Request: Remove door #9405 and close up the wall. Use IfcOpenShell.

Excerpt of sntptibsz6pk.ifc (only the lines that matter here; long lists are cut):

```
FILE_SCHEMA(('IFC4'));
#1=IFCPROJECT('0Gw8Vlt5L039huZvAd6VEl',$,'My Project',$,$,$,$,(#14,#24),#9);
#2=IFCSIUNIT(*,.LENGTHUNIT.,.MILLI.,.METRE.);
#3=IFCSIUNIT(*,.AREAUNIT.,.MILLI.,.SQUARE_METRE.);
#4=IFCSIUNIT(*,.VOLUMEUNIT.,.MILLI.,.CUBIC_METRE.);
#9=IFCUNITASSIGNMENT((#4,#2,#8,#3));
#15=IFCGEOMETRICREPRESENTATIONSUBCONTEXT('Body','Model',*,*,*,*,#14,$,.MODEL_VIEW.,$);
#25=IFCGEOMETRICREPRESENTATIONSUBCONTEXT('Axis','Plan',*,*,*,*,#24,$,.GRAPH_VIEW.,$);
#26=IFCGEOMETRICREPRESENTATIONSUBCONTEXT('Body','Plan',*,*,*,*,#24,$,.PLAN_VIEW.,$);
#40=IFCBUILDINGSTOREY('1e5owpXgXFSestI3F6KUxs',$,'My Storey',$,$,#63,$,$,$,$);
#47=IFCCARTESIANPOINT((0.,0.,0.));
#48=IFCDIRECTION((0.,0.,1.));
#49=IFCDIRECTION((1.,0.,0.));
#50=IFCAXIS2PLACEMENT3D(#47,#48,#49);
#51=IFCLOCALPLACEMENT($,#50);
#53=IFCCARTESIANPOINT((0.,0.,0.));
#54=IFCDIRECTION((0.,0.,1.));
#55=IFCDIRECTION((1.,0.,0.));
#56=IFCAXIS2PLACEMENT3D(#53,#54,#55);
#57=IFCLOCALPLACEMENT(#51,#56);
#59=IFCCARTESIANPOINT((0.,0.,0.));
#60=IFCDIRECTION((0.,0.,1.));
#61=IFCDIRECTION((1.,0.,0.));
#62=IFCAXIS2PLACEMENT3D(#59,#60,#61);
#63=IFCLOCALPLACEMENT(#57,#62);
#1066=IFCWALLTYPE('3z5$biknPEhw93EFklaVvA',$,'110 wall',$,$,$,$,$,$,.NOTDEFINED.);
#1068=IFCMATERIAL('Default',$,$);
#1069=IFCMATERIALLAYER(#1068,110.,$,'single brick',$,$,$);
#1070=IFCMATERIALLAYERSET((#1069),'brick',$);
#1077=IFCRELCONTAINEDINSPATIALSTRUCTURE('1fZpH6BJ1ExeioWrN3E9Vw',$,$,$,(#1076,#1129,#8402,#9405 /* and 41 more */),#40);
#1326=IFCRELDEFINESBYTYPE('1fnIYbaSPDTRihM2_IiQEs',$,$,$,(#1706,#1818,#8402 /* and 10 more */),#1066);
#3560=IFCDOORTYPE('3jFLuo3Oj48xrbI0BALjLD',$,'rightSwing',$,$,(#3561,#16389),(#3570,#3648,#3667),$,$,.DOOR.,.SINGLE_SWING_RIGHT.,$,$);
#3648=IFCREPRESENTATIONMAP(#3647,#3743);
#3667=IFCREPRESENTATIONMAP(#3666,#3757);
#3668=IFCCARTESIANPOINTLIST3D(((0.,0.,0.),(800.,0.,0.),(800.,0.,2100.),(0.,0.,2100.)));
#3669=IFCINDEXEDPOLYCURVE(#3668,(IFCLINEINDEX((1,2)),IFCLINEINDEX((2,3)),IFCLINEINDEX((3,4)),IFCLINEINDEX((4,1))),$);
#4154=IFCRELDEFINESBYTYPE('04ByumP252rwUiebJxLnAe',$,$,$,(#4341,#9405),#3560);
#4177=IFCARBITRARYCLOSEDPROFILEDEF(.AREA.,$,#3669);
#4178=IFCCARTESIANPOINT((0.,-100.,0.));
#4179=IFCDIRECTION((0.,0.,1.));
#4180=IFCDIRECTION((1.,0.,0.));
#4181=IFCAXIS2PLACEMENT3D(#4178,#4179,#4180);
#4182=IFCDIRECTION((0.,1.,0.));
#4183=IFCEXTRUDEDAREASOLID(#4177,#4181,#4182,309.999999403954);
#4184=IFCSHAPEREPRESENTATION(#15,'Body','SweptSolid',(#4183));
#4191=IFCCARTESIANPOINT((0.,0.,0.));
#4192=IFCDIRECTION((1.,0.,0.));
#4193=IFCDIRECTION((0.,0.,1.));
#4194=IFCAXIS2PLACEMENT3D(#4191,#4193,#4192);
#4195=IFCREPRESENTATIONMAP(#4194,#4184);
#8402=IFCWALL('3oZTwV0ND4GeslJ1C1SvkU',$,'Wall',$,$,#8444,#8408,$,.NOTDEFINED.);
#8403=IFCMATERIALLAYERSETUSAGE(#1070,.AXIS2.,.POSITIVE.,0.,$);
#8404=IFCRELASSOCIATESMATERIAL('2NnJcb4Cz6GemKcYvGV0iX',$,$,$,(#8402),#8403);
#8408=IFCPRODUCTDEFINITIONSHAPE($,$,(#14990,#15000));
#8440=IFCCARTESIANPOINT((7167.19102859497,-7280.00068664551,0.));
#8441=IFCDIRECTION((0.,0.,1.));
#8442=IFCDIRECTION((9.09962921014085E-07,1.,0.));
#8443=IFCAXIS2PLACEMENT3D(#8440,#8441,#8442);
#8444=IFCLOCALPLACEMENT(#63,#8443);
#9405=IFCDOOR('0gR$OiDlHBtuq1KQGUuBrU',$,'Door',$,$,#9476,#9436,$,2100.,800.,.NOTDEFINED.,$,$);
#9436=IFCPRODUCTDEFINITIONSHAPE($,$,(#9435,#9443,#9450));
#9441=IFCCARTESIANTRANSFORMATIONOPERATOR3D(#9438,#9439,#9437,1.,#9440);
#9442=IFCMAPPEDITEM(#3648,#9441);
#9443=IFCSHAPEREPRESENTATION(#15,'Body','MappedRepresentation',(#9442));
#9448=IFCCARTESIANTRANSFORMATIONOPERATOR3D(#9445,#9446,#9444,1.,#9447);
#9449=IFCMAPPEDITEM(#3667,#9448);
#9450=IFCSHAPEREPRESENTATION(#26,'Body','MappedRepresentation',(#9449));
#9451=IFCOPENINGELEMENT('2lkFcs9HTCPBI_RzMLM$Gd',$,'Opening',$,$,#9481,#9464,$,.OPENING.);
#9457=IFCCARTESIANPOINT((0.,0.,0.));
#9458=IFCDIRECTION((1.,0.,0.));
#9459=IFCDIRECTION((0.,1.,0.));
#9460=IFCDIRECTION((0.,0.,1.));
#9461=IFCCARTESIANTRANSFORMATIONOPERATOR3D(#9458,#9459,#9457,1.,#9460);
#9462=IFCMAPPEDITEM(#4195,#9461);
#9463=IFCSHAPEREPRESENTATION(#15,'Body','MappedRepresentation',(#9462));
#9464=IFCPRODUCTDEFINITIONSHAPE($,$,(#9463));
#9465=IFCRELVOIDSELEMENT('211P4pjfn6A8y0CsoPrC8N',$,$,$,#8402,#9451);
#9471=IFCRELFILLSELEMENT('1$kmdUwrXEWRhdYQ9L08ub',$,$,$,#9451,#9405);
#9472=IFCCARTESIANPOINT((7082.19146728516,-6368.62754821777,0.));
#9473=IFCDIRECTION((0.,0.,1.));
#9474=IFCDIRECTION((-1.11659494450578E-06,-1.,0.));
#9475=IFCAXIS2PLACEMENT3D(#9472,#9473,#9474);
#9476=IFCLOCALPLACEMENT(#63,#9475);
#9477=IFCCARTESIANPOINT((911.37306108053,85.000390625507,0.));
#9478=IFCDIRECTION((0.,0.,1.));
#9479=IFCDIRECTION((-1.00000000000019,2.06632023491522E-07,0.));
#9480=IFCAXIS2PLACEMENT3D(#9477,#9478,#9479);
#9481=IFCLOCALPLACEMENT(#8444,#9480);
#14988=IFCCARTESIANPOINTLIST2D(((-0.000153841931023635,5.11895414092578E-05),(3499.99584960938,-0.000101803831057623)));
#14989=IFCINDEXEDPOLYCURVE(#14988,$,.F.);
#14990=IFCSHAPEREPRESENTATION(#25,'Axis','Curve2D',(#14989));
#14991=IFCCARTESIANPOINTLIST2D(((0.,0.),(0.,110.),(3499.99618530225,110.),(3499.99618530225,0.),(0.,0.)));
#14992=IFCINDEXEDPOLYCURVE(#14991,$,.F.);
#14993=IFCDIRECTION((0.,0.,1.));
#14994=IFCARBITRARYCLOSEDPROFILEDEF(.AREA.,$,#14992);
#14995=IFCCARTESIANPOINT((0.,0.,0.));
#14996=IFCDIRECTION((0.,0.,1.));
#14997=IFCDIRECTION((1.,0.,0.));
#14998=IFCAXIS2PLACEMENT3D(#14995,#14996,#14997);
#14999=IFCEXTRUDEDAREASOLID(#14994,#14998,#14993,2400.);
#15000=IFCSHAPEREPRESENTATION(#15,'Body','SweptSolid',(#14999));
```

```python
import ifcopenshell
import ifcopenshell.api.feature
import ifcopenshell.api.root
import ifcopenshell.geom
import ifcopenshell.util.shape

model = ifcopenshell.open("sntptibsz6pk.ifc")
settings = ifcopenshell.geom.settings()


def volume(element):
    """Net volume in cubic metres, openings subtracted."""
    shape = ifcopenshell.geom.create_shape(settings, element)
    return ifcopenshell.util.shape.get_volume(shape.geometry)


door = model.by_guid("0gR$OiDlHBtuq1KQGUuBrU")
opening = door.FillsVoids[0].RelatingOpeningElement
wall = opening.VoidsElements[0].RelatingBuildingElement
before = volume(wall)

ifcopenshell.api.root.remove_product(model, product=door)
ifcopenshell.api.feature.remove_feature(model, feature=opening)

after = volume(wall)

print(f"wall volume {before:.3f} -> {after:.3f} m3")

model.write("sntptibsz6pk_rev.ifc")
```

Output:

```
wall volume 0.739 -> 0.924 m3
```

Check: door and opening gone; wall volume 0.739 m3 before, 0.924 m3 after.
